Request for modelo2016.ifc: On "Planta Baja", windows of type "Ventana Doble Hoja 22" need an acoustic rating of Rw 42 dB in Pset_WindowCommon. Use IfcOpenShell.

First a look at what the model holds.

```python
import ifcopenshell
import ifcopenshell.util.element

model = ifcopenshell.open("modelo2016.ifc")
print(model.schema)
storey = next(s for s in model.by_type("IfcBuildingStorey") if s.Name == "Planta Baja")
windows = [e for e in ifcopenshell.util.element.get_decomposition(storey) if e.is_a("IfcWindow")]
seen = {}
for e in windows:
    element_type = ifcopenshell.util.element.get_type(e)
    key = (element_type.Name if element_type != e and element_type else None, ifcopenshell.util.element.get_pset(e, "Pset_WindowCommon", "AcousticRating"))
    seen[key] = seen.get(key, 0) + 1
for (name, value), count in sorted(seen.items(), key=str):
    print(count, "x", name, "|", value)
```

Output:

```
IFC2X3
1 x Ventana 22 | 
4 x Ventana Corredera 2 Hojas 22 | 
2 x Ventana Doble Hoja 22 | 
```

```python
import ifcopenshell
import ifcopenshell.api.pset
import ifcopenshell.util.element

model = ifcopenshell.open("modelo2016.ifc")

storey = next(s for s in model.by_type("IfcBuildingStorey") if s.Name == "Planta Baja")
windows = [e for e in ifcopenshell.util.element.get_decomposition(storey) if e.is_a("IfcWindow")]

count = 0
for e in windows:
    element_type = ifcopenshell.util.element.get_type(e)
    if element_type in (None, e) or element_type.Name != "Ventana Doble Hoja 22":
        continue
    # add_pset returns the element's existing set when there is one.
    pset = ifcopenshell.api.pset.add_pset(model, product=e, name="Pset_WindowCommon")
    ifcopenshell.api.pset.edit_pset(model, pset=pset, properties={"AcousticRating": "Rw 42 dB"})
    count += 1

print(count, "windows updated")

model.write("modelo2016_v2.ifc")
```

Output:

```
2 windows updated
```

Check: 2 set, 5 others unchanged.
